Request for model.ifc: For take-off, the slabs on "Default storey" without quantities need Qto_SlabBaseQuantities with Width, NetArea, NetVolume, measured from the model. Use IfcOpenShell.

First a look at what the model holds.

```python
import ifcopenshell
import ifcopenshell.util.element
import ifcopenshell.util.unit

model = ifcopenshell.open("model.ifc")
print(model.schema)
for unit_type in ("LENGTHUNIT", "AREAUNIT", "VOLUMEUNIT"):
    print(unit_type, ifcopenshell.util.unit.calculate_unit_scale(model, unit_type))
storey = next(s for s in model.by_type("IfcBuildingStorey") if s.Name == "Default storey")
slabs = [e for e in ifcopenshell.util.element.get_decomposition(storey) if e.is_a("IfcSlab")]
for e in sorted(slabs, key=lambda e: e.id()):
    print(e.id(), e.is_a(), e.Name, list(ifcopenshell.util.element.get_psets(e, qtos_only=True)), sep=" | ")
```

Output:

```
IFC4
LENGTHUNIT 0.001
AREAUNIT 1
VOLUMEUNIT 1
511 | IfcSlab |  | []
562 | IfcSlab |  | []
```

```python
import ifcopenshell
import ifcopenshell.api.pset
import ifcopenshell.geom
import ifcopenshell.util.element
import ifcopenshell.util.shape
import ifcopenshell.util.unit

model = ifcopenshell.open("model.ifc")
unit_scale = ifcopenshell.util.unit.calculate_unit_scale(model)
area_scale = ifcopenshell.util.unit.calculate_unit_scale(model, "AREAUNIT")
volume_scale = ifcopenshell.util.unit.calculate_unit_scale(model, "VOLUMEUNIT")
settings = ifcopenshell.geom.settings()

storey = next(s for s in model.by_type("IfcBuildingStorey") if s.Name == "Default storey")
slabs = [e for e in ifcopenshell.util.element.get_decomposition(storey) if e.is_a("IfcSlab")]

for e in sorted(slabs, key=lambda e: e.id()):
    if ifcopenshell.util.element.get_psets(e, qtos_only=True, should_inherit=False):
        continue
    # Geometry comes back in metres, in the element's own axes.
    shape = ifcopenshell.geom.create_shape(settings, e)
    values = {
        "Width": ifcopenshell.util.shape.get_z(shape.geometry) / unit_scale,
        "NetArea": ifcopenshell.util.shape.get_footprint_area(shape.geometry) / area_scale,
        "NetVolume": ifcopenshell.util.shape.get_volume(shape.geometry) / volume_scale,
    }
    qto = ifcopenshell.api.pset.add_qto(model, product=e, name="Qto_SlabBaseQuantities")
    ifcopenshell.api.pset.edit_qto(model, qto=qto, properties=values)
    print(e.id(), {k: round(v, 3) for k, v in values.items()})

model.write("model_rev.ifc")
```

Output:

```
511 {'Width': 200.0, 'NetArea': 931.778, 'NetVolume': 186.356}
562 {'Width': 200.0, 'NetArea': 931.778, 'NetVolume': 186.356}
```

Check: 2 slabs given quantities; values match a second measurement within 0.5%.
